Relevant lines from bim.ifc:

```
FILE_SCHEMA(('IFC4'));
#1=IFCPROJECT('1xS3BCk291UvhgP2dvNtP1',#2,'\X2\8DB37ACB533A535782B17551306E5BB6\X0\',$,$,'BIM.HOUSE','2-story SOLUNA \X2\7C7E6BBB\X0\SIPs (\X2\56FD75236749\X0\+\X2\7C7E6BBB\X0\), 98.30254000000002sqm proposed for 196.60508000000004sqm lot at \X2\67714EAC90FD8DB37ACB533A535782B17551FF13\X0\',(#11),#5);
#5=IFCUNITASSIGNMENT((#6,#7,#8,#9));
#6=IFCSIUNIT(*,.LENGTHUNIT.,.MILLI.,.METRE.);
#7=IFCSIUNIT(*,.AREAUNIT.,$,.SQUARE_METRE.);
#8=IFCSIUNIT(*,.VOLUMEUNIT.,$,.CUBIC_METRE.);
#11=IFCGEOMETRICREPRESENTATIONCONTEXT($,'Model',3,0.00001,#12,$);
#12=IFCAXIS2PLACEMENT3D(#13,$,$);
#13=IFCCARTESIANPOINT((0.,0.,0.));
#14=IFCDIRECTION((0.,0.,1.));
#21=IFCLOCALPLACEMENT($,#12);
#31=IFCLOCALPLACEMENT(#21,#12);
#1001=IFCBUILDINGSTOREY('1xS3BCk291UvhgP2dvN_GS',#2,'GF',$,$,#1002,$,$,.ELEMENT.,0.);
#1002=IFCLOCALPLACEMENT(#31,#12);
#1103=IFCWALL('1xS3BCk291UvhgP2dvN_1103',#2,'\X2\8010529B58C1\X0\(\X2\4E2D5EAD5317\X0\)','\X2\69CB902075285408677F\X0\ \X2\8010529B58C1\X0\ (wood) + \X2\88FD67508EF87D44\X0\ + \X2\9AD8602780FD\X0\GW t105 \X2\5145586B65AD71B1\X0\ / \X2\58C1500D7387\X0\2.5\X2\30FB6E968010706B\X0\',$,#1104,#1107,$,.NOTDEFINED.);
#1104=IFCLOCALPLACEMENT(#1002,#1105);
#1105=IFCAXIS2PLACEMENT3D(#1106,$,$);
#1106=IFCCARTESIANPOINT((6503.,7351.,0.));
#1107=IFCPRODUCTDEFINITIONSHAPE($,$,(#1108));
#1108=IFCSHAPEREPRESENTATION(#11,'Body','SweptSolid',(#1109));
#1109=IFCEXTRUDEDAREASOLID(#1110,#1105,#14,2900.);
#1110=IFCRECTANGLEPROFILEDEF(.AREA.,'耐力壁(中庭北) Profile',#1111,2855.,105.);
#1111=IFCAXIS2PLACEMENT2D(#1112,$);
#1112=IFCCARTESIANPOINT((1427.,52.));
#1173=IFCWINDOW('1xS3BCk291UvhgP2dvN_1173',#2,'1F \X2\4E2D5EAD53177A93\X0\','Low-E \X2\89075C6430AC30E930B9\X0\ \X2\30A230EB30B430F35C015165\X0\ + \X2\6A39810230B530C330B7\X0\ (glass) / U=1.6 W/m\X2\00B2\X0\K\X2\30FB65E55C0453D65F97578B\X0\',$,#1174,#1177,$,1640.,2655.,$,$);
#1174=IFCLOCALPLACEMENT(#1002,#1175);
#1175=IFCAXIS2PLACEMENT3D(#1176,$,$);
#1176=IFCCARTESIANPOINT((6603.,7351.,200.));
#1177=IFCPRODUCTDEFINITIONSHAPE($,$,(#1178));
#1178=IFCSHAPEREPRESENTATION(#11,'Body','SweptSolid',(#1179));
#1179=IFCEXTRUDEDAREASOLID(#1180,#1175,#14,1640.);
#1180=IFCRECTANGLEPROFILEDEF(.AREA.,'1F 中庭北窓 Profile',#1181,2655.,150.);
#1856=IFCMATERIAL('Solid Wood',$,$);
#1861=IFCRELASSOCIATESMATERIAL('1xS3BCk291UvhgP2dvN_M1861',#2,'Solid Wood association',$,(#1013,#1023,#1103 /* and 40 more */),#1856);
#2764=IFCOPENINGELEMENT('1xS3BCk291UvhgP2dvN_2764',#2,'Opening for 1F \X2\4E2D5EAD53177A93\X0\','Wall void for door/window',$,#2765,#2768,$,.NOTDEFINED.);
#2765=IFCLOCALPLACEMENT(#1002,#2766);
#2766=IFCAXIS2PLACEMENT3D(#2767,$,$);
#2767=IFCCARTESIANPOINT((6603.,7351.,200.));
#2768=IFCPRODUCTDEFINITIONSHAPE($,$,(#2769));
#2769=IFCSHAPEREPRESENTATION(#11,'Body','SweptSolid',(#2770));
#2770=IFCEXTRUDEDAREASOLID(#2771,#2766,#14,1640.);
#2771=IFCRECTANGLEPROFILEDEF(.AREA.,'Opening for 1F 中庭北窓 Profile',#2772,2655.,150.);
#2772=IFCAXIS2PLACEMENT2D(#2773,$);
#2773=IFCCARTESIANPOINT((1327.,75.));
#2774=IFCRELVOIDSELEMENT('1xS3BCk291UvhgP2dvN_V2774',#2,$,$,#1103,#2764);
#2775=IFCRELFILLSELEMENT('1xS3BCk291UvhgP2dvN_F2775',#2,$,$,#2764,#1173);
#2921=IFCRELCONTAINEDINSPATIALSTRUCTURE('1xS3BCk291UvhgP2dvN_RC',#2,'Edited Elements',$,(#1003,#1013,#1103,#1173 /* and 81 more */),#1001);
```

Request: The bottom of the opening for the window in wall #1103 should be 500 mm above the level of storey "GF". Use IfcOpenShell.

```python
import numpy as np
import ifcopenshell
import ifcopenshell.api.geometry
import ifcopenshell.geom
import ifcopenshell.util.element
import ifcopenshell.util.placement
import ifcopenshell.util.shape
import ifcopenshell.util.unit

model = ifcopenshell.open("bim.ifc")
unit_scale = ifcopenshell.util.unit.calculate_unit_scale(model)

window = model.by_id(1173)
opening = window.FillsVoids[0].RelatingOpeningElement
storey = ifcopenshell.util.element.get_container(window, ifc_class="IfcBuildingStorey")
level = ifcopenshell.util.placement.get_local_placement(storey.ObjectPlacement)[2, 3]

# The opening's origin need not be at the sill, so measure its lowest point.
shape = ifcopenshell.geom.create_shape(ifcopenshell.geom.settings(), opening)
bottom = ifcopenshell.util.shape.get_shape_bottom_elevation(shape, shape.geometry) / unit_scale
dz = level + 0.5 / unit_scale - bottom

shift = np.array([0.0, 0.0, dz])
# The window is not placed relative to its opening, so move both.
for product in (opening, window):
    matrix = ifcopenshell.util.placement.get_local_placement(product.ObjectPlacement)
    matrix[:3, 3] += shift
    ifcopenshell.api.geometry.edit_object_placement(model, product=product, matrix=matrix, is_si=False)

print(f"moved by {dz * unit_scale:+.3f} m")

model.write("bim_v2.ifc")
```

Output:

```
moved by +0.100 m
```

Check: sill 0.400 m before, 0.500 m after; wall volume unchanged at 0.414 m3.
